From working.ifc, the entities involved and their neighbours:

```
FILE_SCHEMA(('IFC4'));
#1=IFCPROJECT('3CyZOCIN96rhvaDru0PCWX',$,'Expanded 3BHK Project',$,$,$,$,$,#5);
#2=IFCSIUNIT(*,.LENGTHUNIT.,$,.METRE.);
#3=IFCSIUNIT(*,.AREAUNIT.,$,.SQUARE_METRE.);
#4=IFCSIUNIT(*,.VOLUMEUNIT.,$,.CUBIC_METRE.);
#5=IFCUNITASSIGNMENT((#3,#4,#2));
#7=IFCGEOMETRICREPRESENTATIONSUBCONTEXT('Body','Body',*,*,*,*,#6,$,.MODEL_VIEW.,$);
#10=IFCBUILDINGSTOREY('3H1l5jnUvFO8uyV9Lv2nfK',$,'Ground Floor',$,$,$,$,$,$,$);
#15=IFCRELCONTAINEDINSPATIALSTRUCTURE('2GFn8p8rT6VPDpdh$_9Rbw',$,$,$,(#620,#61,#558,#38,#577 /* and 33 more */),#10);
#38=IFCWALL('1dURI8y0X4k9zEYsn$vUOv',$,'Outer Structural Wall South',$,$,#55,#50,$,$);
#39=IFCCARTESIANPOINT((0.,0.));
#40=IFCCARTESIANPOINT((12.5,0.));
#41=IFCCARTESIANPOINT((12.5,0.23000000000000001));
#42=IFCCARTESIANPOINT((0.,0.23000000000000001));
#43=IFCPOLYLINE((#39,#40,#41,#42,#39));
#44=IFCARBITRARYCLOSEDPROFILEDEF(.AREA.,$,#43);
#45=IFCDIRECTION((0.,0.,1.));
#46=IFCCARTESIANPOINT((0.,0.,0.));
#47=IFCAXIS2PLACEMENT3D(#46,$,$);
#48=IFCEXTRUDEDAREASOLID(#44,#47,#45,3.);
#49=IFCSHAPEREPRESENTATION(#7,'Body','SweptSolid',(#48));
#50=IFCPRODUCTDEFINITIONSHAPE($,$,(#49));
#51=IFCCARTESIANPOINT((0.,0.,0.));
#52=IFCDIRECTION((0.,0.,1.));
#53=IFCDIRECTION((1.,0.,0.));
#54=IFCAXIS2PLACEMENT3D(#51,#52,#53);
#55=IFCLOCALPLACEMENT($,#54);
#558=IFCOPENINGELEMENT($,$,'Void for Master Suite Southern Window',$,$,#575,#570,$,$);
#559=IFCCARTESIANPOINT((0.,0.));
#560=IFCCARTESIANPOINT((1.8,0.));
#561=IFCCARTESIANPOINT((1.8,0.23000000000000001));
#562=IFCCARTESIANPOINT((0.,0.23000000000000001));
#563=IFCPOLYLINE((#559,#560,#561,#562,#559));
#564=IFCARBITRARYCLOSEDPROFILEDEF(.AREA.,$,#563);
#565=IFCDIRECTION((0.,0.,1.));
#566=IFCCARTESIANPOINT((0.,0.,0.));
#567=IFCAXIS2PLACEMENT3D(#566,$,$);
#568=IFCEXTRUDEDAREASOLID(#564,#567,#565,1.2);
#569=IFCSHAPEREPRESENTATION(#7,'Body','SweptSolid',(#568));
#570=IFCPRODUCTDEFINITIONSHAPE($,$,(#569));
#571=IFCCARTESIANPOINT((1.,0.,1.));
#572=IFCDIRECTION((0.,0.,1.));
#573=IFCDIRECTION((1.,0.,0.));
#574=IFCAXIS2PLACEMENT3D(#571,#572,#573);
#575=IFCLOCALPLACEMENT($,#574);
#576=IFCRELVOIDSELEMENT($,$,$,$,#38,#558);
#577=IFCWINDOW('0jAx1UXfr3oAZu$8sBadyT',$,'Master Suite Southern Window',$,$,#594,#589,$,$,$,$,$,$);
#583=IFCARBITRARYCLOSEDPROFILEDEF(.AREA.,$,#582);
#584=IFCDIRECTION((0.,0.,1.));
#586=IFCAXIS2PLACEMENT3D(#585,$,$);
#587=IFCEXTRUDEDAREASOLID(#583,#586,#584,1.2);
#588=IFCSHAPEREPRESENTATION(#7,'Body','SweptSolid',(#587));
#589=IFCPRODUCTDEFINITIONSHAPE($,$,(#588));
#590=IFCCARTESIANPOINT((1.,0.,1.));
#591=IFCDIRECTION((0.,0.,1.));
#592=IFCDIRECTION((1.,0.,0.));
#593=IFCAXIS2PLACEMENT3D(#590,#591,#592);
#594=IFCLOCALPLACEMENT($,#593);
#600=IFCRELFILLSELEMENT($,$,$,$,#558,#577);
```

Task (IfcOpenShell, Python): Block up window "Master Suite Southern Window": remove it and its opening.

```python
import ifcopenshell
import ifcopenshell.api.feature
import ifcopenshell.api.root
import ifcopenshell.geom
import ifcopenshell.util.shape

model = ifcopenshell.open("working.ifc")
settings = ifcopenshell.geom.settings()


def volume(element):
    """Net volume in cubic metres, openings subtracted."""
    shape = ifcopenshell.geom.create_shape(settings, element)
    return ifcopenshell.util.shape.get_volume(shape.geometry)


window = model.by_guid("0jAx1UXfr3oAZu$8sBadyT")
opening = window.FillsVoids[0].RelatingOpeningElement
wall = opening.VoidsElements[0].RelatingBuildingElement
before = volume(wall)

ifcopenshell.api.root.remove_product(model, product=window)
ifcopenshell.api.feature.remove_feature(model, feature=opening)

after = volume(wall)

print(f"wall volume {before:.3f} -> {after:.3f} m3")

model.write("working_updated.ifc")
```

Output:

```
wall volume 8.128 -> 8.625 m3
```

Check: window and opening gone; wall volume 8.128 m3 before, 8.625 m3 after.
